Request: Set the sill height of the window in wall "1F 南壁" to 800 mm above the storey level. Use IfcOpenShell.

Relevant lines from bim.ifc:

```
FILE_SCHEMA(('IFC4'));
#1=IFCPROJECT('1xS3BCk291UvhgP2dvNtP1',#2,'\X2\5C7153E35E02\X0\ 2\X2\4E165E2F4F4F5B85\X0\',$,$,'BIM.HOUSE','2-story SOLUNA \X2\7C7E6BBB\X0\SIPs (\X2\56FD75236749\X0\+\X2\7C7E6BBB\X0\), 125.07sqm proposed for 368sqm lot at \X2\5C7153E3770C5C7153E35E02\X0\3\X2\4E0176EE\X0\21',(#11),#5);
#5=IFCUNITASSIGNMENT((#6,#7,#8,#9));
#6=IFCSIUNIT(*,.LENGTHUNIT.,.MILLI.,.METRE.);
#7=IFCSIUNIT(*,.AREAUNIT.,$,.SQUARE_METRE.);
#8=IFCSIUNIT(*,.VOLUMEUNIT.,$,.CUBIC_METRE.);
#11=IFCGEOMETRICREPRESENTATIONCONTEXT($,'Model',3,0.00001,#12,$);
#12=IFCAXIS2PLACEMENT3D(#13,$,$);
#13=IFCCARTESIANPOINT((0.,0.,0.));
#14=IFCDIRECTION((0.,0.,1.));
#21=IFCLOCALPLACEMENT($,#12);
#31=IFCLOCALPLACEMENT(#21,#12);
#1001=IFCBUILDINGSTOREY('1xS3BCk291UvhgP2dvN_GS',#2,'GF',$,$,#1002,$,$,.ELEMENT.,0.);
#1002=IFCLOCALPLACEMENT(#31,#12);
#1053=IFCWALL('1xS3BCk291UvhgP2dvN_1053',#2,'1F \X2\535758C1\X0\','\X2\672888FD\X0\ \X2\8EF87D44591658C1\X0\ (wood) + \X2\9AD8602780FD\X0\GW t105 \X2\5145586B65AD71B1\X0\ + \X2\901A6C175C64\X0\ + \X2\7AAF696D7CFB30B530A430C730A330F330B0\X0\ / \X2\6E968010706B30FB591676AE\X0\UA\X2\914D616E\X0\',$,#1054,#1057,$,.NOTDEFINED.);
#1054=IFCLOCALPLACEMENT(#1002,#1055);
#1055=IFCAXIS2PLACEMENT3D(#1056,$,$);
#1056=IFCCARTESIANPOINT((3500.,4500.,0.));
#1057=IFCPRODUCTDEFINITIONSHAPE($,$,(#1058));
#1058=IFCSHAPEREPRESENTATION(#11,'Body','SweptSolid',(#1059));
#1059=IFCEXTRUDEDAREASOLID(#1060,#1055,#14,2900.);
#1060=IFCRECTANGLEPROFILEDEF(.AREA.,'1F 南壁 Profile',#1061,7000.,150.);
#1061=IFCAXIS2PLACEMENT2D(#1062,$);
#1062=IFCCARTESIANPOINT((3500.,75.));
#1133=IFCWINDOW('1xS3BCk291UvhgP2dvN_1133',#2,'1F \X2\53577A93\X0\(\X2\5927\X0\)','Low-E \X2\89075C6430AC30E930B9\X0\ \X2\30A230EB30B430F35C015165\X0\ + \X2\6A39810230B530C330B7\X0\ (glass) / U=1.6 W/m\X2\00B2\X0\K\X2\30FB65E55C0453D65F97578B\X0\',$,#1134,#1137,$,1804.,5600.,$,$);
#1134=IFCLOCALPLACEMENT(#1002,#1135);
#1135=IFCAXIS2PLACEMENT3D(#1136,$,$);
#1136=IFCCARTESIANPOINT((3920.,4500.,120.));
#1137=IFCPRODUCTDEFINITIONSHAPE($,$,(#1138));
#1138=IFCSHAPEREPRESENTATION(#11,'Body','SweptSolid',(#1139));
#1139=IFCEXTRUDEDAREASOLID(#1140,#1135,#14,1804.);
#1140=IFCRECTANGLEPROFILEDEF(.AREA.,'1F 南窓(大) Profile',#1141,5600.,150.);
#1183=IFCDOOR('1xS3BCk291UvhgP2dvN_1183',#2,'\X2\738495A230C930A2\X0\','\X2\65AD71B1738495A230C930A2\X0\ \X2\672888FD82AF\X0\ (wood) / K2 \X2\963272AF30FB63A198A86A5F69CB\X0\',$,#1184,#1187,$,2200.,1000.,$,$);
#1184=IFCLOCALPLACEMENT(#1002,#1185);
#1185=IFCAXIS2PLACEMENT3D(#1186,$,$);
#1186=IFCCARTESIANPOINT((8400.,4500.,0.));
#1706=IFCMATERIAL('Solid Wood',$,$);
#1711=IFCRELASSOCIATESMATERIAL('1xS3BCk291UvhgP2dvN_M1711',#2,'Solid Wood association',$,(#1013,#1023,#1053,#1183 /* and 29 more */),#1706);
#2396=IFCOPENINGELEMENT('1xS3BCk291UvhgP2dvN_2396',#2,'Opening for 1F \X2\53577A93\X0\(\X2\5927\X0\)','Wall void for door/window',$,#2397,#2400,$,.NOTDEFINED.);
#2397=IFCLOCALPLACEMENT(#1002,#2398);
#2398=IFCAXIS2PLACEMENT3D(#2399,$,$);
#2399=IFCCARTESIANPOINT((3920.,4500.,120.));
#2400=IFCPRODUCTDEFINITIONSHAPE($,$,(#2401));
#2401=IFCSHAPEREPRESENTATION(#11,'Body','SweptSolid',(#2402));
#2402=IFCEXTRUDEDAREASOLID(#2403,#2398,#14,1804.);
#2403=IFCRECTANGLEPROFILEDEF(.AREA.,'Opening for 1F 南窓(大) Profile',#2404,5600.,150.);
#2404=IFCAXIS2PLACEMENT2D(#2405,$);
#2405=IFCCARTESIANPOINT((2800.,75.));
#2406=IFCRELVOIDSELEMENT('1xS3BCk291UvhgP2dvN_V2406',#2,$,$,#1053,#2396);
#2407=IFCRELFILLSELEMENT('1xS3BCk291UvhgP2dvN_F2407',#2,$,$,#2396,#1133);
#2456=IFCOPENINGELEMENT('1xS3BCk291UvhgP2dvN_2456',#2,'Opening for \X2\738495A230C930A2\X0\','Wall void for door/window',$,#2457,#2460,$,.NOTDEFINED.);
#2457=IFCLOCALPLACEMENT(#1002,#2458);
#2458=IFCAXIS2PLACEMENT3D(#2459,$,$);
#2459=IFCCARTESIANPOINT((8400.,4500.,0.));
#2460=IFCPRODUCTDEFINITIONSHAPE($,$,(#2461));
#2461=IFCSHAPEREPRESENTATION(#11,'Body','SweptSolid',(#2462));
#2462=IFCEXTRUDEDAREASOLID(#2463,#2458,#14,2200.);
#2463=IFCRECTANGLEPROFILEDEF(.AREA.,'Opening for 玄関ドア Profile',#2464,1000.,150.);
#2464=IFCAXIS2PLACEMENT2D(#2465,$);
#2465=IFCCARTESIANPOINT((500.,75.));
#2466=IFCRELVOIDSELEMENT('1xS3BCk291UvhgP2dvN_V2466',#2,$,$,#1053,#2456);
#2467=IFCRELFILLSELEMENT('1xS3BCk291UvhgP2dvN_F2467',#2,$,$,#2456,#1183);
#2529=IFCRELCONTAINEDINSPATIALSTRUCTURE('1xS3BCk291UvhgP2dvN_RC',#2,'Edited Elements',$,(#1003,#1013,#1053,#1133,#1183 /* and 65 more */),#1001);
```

```python
import numpy as np
import ifcopenshell
import ifcopenshell.api.geometry
import ifcopenshell.geom
import ifcopenshell.util.element
import ifcopenshell.util.placement
import ifcopenshell.util.shape
import ifcopenshell.util.unit

model = ifcopenshell.open("bim.ifc")
unit_scale = ifcopenshell.util.unit.calculate_unit_scale(model)

window = model.by_id(1133)
opening = window.FillsVoids[0].RelatingOpeningElement
storey = ifcopenshell.util.element.get_container(window, ifc_class="IfcBuildingStorey")
level = ifcopenshell.util.placement.get_local_placement(storey.ObjectPlacement)[2, 3]

# The opening's origin need not be at the sill, so measure its lowest point.
shape = ifcopenshell.geom.create_shape(ifcopenshell.geom.settings(), opening)
bottom = ifcopenshell.util.shape.get_shape_bottom_elevation(shape, shape.geometry) / unit_scale
dz = level + 800.0 - bottom

shift = np.array([0.0, 0.0, dz])
# The window is not placed relative to its opening, so move both.
for product in (opening, window):
    matrix = ifcopenshell.util.placement.get_local_placement(product.ObjectPlacement)
    matrix[:3, 3] += shift
    ifcopenshell.api.geometry.edit_object_placement(model, product=product, matrix=matrix, is_si=False)

print(f"moved by {dz * unit_scale:+.3f} m")

model.write("bim-out.ifc")
```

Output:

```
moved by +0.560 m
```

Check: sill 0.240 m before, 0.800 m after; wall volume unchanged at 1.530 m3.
